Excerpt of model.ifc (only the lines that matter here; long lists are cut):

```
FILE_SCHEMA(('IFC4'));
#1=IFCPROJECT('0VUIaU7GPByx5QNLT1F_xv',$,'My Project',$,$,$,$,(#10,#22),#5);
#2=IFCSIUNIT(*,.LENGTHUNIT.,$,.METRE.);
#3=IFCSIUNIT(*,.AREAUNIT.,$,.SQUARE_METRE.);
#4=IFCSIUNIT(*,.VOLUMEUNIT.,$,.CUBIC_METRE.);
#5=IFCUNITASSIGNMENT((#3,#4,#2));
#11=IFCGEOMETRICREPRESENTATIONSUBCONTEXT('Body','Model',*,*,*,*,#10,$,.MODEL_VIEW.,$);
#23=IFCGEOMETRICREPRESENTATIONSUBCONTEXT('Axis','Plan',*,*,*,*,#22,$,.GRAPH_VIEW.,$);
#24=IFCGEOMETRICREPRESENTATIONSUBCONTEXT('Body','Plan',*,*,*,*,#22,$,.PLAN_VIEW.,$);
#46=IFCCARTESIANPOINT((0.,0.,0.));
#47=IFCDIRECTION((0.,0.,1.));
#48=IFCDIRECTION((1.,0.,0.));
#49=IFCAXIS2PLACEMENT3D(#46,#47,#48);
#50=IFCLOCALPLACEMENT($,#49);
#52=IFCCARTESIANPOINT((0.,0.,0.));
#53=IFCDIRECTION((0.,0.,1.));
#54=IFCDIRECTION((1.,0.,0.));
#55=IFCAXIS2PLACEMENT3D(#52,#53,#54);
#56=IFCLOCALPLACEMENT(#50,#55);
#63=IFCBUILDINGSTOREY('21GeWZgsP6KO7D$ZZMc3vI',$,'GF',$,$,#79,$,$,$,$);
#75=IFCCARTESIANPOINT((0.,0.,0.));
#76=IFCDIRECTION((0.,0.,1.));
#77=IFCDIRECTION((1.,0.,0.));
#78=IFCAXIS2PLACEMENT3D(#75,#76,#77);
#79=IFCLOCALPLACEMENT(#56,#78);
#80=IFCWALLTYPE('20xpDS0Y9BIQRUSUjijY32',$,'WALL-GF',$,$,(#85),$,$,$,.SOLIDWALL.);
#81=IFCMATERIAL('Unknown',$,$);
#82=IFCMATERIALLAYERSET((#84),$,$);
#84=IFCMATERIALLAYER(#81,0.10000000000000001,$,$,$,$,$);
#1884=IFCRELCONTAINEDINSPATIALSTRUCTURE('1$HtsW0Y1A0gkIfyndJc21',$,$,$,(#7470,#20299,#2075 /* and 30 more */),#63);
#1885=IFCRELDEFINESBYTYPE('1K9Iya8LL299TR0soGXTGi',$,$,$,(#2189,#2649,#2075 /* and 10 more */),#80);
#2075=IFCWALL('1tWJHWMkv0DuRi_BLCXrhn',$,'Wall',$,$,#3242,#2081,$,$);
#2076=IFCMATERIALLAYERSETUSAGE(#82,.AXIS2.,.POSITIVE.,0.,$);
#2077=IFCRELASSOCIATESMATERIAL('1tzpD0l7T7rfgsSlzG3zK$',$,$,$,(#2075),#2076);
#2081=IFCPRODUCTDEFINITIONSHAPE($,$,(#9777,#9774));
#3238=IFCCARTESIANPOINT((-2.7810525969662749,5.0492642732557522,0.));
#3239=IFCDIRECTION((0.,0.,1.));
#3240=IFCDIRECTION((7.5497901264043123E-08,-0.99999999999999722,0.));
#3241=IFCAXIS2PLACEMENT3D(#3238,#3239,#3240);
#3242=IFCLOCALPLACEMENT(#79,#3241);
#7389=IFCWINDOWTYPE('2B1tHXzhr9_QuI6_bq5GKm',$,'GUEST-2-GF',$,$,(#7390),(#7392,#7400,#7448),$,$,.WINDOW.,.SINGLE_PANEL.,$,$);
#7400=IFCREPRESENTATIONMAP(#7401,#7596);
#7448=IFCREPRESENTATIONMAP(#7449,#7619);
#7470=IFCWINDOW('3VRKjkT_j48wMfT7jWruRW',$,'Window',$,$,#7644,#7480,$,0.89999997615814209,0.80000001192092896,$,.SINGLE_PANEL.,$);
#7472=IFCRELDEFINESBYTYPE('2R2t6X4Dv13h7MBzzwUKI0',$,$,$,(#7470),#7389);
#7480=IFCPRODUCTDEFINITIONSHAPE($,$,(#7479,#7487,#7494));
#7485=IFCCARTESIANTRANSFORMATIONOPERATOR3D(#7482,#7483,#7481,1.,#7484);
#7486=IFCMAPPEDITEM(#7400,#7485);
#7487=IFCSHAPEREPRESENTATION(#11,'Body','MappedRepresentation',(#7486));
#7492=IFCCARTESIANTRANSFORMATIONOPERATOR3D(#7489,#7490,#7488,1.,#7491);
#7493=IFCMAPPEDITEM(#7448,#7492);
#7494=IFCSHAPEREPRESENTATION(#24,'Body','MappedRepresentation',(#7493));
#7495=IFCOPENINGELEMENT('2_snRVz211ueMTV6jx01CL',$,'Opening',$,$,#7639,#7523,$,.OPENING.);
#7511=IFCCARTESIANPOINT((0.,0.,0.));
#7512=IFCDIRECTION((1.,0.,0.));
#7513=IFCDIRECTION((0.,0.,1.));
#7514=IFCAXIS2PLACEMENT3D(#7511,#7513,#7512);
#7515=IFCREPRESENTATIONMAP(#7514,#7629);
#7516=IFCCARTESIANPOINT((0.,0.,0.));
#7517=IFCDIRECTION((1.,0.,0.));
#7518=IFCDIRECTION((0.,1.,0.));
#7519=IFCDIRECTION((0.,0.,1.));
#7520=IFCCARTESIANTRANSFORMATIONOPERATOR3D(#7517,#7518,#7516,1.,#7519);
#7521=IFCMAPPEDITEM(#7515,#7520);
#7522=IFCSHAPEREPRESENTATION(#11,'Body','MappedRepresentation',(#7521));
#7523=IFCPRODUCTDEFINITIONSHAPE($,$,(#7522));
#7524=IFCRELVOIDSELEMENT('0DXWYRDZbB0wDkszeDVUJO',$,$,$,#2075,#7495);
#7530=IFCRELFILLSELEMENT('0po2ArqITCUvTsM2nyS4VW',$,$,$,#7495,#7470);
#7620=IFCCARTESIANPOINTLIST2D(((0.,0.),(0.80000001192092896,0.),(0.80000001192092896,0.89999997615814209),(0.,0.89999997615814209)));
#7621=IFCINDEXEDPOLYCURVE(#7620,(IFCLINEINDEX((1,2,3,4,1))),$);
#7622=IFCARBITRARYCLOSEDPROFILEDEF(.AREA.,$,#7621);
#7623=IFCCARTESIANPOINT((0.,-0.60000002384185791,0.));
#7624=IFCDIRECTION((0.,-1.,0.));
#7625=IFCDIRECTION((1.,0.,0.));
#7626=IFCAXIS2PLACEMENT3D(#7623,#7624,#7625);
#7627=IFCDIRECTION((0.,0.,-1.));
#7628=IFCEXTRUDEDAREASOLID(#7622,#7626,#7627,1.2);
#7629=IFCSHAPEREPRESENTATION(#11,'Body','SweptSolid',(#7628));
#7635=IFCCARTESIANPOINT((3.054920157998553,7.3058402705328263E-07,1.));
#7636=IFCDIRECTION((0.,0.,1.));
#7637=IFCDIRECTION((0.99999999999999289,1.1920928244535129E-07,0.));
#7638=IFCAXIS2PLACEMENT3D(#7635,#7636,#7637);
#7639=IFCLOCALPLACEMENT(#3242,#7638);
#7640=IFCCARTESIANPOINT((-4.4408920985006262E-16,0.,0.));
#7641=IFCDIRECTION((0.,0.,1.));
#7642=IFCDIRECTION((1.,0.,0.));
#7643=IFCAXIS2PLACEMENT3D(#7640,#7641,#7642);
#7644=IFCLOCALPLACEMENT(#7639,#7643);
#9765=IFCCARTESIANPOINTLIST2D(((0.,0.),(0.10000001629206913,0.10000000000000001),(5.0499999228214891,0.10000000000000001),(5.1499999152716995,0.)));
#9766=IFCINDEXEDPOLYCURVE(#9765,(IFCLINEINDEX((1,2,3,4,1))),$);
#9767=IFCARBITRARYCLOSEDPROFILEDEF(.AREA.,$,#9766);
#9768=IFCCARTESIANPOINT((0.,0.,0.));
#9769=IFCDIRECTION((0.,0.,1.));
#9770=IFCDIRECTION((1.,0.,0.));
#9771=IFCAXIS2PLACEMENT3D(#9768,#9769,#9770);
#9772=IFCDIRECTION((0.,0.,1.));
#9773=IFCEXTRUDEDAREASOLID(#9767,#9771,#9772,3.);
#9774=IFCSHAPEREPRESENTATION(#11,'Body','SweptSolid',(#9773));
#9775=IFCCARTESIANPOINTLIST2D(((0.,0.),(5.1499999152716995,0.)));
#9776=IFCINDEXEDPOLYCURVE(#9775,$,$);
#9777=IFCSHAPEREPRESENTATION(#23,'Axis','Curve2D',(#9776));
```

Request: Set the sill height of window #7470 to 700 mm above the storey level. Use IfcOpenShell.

```python
import numpy as np
import ifcopenshell
import ifcopenshell.api.geometry
import ifcopenshell.geom
import ifcopenshell.util.element
import ifcopenshell.util.placement
import ifcopenshell.util.shape
import ifcopenshell.util.unit

model = ifcopenshell.open("model.ifc")
unit_scale = ifcopenshell.util.unit.calculate_unit_scale(model)

window = model.by_guid("3VRKjkT_j48wMfT7jWruRW")
opening = window.FillsVoids[0].RelatingOpeningElement
storey = ifcopenshell.util.element.get_container(window, ifc_class="IfcBuildingStorey")
level = ifcopenshell.util.placement.get_local_placement(storey.ObjectPlacement)[2, 3]

# The opening's origin need not be at the sill, so measure its lowest point.
shape = ifcopenshell.geom.create_shape(ifcopenshell.geom.settings(), opening)
bottom = ifcopenshell.util.shape.get_shape_bottom_elevation(shape, shape.geometry) / unit_scale
dz = level + 0.7 / unit_scale - bottom

shift = np.array([0.0, 0.0, dz])
# The window is placed relative to its opening, so it follows when the opening moves.
matrix = ifcopenshell.util.placement.get_local_placement(opening.ObjectPlacement)
matrix[:3, 3] += shift
ifcopenshell.api.geometry.edit_object_placement(
    model, product=opening, matrix=matrix, is_si=False, should_transform_children=True
)

print(f"moved by {dz * unit_scale:+.3f} m")

model.write("model_updated.ifc")
```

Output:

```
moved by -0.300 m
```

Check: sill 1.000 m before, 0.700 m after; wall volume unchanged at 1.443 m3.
